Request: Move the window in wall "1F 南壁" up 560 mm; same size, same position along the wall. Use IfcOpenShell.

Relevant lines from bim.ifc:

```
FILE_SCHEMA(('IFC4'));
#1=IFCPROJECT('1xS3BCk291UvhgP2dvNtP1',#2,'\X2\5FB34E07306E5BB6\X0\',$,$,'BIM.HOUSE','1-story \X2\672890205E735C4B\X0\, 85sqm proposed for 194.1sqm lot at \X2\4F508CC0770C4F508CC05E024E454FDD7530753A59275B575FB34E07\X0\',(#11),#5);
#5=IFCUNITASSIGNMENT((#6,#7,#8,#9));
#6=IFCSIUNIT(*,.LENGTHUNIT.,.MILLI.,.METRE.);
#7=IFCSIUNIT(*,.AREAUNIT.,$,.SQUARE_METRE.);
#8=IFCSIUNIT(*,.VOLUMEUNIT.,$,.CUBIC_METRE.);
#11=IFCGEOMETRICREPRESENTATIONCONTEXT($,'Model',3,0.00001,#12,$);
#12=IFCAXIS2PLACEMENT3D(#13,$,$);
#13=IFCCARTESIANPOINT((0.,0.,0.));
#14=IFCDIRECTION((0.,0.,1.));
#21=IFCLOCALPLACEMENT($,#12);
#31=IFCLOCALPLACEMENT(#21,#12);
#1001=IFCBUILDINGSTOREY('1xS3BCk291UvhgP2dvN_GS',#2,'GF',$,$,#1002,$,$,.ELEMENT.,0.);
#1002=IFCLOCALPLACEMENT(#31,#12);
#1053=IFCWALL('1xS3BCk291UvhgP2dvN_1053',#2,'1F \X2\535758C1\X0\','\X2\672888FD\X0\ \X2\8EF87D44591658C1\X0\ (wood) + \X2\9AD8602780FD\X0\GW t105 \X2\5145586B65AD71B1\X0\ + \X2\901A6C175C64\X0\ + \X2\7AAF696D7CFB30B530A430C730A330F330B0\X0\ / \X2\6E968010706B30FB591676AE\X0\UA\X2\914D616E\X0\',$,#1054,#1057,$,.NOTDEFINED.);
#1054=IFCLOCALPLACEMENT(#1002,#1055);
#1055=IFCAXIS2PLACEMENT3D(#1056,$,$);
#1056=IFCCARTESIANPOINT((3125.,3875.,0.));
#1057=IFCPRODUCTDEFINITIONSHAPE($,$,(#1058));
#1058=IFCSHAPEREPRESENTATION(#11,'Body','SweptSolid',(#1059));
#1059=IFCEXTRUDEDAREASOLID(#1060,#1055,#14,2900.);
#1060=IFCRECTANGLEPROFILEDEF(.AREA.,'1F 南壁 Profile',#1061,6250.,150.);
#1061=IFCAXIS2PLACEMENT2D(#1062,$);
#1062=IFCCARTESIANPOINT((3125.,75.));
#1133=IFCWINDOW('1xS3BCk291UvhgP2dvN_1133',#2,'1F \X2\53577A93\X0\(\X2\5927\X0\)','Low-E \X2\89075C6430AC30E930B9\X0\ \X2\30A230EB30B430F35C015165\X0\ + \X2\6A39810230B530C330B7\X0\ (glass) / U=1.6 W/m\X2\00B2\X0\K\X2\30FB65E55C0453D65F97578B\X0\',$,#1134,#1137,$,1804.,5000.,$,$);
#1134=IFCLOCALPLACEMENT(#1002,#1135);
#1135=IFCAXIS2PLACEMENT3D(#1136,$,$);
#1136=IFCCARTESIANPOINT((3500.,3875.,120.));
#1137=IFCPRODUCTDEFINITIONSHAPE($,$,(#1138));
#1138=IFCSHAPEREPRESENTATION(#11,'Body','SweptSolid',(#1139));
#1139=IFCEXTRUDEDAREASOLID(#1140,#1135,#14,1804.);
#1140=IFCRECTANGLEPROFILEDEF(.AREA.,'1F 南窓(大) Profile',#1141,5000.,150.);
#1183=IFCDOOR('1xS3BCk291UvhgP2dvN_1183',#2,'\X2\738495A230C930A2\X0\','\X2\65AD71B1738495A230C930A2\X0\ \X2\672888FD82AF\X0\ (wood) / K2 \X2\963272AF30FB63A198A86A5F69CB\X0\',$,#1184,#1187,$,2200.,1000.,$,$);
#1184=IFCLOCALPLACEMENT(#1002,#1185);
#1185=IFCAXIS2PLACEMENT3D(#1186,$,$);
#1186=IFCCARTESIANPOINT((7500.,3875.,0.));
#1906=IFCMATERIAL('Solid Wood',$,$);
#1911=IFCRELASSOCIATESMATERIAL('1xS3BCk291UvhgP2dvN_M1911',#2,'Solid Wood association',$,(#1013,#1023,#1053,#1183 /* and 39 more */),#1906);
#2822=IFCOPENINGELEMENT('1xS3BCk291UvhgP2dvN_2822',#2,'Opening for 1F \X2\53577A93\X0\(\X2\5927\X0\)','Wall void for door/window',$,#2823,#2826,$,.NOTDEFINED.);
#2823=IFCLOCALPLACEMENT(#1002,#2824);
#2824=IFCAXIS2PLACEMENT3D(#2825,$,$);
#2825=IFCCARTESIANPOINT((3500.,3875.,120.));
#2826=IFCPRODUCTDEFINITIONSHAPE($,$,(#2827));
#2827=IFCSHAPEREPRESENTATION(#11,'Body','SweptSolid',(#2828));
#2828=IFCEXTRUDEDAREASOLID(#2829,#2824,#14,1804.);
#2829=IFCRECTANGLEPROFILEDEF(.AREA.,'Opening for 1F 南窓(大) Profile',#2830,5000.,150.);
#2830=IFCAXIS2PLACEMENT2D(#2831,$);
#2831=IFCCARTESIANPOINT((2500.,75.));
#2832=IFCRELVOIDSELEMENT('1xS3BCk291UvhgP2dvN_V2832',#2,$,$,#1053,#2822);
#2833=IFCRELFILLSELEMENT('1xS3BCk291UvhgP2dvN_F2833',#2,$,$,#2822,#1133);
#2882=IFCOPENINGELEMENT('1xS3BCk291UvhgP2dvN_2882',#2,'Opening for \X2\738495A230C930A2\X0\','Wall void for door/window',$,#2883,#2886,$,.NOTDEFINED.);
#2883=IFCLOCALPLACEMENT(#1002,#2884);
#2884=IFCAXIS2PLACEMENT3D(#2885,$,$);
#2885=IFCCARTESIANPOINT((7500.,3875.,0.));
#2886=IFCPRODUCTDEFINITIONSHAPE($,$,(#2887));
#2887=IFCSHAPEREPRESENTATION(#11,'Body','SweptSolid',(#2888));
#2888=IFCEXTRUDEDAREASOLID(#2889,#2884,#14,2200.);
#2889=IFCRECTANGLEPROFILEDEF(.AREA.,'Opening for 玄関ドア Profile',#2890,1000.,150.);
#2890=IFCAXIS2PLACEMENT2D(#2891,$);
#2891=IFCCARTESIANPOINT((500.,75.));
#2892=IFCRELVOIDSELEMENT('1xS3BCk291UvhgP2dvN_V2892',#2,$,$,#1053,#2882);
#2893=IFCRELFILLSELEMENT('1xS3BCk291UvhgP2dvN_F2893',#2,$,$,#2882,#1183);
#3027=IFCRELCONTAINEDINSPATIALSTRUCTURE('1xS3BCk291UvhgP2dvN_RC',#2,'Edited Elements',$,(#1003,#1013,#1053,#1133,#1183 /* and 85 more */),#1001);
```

```python
import numpy as np
import ifcopenshell
import ifcopenshell.api.geometry
import ifcopenshell.util.placement
import ifcopenshell.util.unit

model = ifcopenshell.open("bim.ifc")
unit_scale = ifcopenshell.util.unit.calculate_unit_scale(model)

window = model.by_id(1133)
opening = window.FillsVoids[0].RelatingOpeningElement
dz = 0.56 / unit_scale

shift = np.array([0.0, 0.0, dz])
# The window is not placed relative to its opening, so move both.
for product in (opening, window):
    matrix = ifcopenshell.util.placement.get_local_placement(product.ObjectPlacement)
    matrix[:3, 3] += shift
    ifcopenshell.api.geometry.edit_object_placement(model, product=product, matrix=matrix, is_si=False)

print(f"moved by {dz * unit_scale:+.3f} m")

model.write("bim_v2.ifc")
```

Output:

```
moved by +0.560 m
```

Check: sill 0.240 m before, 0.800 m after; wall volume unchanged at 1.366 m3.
